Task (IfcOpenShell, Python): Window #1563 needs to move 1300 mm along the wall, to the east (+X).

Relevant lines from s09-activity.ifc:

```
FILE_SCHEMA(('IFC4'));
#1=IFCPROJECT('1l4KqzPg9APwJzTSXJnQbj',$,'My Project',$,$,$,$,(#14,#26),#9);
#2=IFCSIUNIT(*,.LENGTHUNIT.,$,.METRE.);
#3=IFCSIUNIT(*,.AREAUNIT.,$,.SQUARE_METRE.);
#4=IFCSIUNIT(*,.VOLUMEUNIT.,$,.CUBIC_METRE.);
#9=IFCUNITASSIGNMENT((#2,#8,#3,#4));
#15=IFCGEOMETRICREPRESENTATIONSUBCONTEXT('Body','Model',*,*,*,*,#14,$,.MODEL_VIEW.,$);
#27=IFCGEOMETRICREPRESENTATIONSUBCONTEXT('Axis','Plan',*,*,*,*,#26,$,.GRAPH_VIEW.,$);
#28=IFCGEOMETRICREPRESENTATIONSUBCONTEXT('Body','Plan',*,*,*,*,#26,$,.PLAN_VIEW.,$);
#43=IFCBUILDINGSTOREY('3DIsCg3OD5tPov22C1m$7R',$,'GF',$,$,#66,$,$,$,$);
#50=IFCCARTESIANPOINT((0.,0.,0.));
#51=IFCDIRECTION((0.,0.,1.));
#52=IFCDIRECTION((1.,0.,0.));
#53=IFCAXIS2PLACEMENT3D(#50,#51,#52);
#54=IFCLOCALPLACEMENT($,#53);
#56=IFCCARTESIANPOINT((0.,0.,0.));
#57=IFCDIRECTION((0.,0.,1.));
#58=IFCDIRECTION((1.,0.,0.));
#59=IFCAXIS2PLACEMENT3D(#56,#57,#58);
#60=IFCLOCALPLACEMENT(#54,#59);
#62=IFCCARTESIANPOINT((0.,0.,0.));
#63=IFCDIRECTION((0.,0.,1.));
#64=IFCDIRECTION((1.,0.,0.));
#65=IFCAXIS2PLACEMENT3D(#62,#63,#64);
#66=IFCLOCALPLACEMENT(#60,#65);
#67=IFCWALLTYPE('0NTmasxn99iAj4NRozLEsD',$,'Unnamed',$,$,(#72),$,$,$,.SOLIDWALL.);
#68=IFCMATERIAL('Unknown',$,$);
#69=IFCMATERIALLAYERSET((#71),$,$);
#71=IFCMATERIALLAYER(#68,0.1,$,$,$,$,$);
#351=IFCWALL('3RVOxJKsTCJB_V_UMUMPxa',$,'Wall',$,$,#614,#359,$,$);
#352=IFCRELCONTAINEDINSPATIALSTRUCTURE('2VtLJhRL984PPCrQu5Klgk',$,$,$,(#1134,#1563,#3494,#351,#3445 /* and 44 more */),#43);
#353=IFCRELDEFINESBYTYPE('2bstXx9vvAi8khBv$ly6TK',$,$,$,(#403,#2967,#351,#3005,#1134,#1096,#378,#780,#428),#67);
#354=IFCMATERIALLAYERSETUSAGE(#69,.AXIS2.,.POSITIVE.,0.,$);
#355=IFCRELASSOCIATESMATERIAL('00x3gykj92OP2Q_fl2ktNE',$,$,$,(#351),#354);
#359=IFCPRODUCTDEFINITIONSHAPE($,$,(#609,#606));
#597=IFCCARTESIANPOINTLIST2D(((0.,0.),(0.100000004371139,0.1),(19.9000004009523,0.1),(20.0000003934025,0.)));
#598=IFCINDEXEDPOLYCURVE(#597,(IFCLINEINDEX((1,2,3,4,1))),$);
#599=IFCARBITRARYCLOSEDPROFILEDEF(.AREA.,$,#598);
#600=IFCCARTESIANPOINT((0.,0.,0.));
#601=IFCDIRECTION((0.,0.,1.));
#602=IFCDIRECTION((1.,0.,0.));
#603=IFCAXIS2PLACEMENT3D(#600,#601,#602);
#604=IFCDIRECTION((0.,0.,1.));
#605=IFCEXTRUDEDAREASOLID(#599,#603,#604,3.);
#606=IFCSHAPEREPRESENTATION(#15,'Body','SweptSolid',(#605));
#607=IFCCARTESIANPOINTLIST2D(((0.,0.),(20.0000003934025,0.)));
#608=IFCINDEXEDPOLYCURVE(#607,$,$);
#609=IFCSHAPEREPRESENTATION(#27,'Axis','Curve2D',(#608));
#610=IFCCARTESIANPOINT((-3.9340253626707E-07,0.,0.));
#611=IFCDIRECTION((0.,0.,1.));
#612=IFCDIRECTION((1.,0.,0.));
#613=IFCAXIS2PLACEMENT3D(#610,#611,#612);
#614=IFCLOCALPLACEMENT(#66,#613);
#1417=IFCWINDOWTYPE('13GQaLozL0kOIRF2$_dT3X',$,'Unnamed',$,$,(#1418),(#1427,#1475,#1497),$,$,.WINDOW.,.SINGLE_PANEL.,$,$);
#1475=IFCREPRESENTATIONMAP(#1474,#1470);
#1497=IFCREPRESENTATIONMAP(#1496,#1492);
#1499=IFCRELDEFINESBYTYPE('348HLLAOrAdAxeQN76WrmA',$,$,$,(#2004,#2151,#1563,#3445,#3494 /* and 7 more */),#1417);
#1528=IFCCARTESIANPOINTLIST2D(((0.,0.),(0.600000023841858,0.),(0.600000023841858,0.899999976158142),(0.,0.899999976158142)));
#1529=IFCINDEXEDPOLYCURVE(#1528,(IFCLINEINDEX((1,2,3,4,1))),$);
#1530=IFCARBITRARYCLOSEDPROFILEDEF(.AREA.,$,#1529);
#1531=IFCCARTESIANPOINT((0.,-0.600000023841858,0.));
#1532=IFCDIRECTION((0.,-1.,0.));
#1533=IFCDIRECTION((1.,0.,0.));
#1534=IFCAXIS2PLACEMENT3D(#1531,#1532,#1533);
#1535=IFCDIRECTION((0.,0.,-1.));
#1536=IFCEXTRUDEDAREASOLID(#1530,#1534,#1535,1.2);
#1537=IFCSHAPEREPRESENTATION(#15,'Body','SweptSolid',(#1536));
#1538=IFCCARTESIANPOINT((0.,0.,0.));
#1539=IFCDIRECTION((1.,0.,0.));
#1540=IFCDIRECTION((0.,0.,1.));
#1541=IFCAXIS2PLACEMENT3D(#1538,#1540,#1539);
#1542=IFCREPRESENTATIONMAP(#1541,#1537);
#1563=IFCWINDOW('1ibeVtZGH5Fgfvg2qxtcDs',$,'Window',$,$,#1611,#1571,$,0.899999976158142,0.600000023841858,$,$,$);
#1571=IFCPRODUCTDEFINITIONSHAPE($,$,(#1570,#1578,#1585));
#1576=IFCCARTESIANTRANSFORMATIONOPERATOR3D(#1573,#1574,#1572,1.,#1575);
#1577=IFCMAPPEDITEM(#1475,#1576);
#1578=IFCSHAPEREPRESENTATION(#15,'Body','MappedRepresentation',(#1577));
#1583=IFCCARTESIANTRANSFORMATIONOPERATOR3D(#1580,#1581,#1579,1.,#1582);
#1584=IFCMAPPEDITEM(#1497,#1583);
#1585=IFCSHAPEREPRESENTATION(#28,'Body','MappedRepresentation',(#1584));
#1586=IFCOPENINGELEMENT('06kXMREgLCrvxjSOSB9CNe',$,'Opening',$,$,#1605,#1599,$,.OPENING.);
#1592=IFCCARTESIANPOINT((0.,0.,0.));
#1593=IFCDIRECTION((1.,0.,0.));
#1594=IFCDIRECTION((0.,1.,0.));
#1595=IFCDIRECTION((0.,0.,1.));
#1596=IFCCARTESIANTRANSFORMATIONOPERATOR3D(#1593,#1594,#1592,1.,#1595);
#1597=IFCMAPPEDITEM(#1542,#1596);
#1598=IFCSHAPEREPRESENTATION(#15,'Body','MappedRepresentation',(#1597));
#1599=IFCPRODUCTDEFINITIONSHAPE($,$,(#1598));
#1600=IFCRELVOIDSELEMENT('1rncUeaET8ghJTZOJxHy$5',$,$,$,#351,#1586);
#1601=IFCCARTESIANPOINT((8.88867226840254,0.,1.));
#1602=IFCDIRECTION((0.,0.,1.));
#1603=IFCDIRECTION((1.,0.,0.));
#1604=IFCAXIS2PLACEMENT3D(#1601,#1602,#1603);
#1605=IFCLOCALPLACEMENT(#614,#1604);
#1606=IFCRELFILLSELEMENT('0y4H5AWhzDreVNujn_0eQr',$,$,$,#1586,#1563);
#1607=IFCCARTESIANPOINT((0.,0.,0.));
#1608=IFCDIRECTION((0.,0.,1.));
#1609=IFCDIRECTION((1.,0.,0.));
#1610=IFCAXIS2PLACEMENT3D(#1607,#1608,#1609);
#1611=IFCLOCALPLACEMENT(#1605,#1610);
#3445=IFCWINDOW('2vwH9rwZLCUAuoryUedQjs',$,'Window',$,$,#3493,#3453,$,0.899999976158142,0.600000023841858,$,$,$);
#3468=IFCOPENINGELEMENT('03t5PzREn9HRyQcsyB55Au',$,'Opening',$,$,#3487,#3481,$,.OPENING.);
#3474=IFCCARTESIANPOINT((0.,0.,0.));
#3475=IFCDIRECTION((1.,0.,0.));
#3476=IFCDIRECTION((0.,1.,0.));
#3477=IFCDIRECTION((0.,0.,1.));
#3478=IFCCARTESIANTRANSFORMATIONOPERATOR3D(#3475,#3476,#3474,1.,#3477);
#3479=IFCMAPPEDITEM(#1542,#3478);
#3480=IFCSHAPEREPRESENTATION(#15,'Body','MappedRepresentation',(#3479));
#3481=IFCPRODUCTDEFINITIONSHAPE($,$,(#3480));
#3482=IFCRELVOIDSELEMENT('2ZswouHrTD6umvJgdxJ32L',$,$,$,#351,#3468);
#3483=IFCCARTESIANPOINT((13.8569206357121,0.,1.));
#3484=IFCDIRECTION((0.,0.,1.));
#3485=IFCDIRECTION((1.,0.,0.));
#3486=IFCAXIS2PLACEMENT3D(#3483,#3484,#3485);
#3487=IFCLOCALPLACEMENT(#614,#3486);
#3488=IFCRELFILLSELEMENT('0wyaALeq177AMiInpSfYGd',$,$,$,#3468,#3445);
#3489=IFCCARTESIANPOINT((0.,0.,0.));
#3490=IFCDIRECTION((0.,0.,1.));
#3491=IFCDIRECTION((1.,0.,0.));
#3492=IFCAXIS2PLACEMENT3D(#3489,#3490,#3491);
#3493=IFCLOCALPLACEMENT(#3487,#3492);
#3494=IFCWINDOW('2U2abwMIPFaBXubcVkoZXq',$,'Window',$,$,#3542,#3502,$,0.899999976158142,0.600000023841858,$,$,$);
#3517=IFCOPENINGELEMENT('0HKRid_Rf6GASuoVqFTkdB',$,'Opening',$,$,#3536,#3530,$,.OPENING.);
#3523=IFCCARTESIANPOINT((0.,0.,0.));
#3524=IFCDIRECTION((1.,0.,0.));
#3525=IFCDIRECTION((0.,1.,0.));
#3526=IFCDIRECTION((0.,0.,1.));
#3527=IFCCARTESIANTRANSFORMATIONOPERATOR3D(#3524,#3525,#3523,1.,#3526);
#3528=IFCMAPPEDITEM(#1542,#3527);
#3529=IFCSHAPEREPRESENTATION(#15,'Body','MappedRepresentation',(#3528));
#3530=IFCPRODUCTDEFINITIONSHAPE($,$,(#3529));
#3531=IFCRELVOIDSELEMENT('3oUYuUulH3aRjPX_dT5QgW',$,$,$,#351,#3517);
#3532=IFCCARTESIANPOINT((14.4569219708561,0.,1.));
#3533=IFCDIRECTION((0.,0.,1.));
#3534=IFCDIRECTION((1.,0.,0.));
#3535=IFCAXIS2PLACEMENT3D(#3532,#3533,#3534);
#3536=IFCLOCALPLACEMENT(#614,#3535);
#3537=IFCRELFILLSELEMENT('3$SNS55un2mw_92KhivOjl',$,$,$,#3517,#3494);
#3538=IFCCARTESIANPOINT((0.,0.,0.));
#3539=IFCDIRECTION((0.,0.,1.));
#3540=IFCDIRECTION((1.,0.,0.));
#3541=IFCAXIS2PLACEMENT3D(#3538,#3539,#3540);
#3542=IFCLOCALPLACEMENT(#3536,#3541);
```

```python
import ifcopenshell
import ifcopenshell.api.geometry
import ifcopenshell.util.placement
import ifcopenshell.util.unit

model = ifcopenshell.open("s09-activity.ifc")
unit_scale = ifcopenshell.util.unit.calculate_unit_scale(model)

window = model.by_guid("1ibeVtZGH5Fgfvg2qxtcDs")
opening = window.FillsVoids[0].RelatingOpeningElement
wall = opening.VoidsElements[0].RelatingBuildingElement

wall_matrix = ifcopenshell.util.placement.get_local_placement(wall.ObjectPlacement)
shift = wall_matrix[:3, 0] * 1.3 / unit_scale
before = ifcopenshell.util.placement.get_local_placement(window.ObjectPlacement)[:3, 3].copy()

# The window is placed relative to its opening, so it follows when the opening moves.
matrix = ifcopenshell.util.placement.get_local_placement(opening.ObjectPlacement)
matrix[:3, 3] += shift
ifcopenshell.api.geometry.edit_object_placement(
    model, product=opening, matrix=matrix, is_si=False, should_transform_children=True
)

after = ifcopenshell.util.placement.get_local_placement(window.ObjectPlacement)[:3, 3]
print("window moved by", (after - before).round(3) + 0.0)

model.write("s09-activity_v2.ifc")
```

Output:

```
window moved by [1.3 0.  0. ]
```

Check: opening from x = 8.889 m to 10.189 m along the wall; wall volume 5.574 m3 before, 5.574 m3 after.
